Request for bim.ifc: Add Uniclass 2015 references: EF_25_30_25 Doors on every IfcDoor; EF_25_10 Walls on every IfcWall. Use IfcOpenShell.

First a look at what the model holds.

```python
import ifcopenshell

model = ifcopenshell.open("bim.ifc")
print(model.schema)
print("classifications:", [c.Name for c in model.by_type("IfcClassification")])
for ifc_class in ("IfcDoor", "IfcRoof", "IfcStair", "IfcWall", "IfcWindow"):
    print(ifc_class, len(model.by_type(ifc_class)))
```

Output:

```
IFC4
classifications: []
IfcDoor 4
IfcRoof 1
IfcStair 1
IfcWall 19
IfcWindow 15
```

```python
import ifcopenshell
import ifcopenshell.api.classification

model = ifcopenshell.open("bim.ifc")

system = ifcopenshell.api.classification.add_classification(model, classification="Uniclass 2015")

codes = {
    "IfcDoor": ("EF_25_30_25", "Doors"),
    "IfcWall": ("EF_25_10", "Walls"),
}
for ifc_class, (code, name) in codes.items():
    products = model.by_type(ifc_class)
    ifcopenshell.api.classification.add_reference(
        model, products=products, classification=system, identification=code, name=name
    )
    print(code, len(products))

model.write("bim_edited.ifc")
```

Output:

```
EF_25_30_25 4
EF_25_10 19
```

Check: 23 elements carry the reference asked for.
